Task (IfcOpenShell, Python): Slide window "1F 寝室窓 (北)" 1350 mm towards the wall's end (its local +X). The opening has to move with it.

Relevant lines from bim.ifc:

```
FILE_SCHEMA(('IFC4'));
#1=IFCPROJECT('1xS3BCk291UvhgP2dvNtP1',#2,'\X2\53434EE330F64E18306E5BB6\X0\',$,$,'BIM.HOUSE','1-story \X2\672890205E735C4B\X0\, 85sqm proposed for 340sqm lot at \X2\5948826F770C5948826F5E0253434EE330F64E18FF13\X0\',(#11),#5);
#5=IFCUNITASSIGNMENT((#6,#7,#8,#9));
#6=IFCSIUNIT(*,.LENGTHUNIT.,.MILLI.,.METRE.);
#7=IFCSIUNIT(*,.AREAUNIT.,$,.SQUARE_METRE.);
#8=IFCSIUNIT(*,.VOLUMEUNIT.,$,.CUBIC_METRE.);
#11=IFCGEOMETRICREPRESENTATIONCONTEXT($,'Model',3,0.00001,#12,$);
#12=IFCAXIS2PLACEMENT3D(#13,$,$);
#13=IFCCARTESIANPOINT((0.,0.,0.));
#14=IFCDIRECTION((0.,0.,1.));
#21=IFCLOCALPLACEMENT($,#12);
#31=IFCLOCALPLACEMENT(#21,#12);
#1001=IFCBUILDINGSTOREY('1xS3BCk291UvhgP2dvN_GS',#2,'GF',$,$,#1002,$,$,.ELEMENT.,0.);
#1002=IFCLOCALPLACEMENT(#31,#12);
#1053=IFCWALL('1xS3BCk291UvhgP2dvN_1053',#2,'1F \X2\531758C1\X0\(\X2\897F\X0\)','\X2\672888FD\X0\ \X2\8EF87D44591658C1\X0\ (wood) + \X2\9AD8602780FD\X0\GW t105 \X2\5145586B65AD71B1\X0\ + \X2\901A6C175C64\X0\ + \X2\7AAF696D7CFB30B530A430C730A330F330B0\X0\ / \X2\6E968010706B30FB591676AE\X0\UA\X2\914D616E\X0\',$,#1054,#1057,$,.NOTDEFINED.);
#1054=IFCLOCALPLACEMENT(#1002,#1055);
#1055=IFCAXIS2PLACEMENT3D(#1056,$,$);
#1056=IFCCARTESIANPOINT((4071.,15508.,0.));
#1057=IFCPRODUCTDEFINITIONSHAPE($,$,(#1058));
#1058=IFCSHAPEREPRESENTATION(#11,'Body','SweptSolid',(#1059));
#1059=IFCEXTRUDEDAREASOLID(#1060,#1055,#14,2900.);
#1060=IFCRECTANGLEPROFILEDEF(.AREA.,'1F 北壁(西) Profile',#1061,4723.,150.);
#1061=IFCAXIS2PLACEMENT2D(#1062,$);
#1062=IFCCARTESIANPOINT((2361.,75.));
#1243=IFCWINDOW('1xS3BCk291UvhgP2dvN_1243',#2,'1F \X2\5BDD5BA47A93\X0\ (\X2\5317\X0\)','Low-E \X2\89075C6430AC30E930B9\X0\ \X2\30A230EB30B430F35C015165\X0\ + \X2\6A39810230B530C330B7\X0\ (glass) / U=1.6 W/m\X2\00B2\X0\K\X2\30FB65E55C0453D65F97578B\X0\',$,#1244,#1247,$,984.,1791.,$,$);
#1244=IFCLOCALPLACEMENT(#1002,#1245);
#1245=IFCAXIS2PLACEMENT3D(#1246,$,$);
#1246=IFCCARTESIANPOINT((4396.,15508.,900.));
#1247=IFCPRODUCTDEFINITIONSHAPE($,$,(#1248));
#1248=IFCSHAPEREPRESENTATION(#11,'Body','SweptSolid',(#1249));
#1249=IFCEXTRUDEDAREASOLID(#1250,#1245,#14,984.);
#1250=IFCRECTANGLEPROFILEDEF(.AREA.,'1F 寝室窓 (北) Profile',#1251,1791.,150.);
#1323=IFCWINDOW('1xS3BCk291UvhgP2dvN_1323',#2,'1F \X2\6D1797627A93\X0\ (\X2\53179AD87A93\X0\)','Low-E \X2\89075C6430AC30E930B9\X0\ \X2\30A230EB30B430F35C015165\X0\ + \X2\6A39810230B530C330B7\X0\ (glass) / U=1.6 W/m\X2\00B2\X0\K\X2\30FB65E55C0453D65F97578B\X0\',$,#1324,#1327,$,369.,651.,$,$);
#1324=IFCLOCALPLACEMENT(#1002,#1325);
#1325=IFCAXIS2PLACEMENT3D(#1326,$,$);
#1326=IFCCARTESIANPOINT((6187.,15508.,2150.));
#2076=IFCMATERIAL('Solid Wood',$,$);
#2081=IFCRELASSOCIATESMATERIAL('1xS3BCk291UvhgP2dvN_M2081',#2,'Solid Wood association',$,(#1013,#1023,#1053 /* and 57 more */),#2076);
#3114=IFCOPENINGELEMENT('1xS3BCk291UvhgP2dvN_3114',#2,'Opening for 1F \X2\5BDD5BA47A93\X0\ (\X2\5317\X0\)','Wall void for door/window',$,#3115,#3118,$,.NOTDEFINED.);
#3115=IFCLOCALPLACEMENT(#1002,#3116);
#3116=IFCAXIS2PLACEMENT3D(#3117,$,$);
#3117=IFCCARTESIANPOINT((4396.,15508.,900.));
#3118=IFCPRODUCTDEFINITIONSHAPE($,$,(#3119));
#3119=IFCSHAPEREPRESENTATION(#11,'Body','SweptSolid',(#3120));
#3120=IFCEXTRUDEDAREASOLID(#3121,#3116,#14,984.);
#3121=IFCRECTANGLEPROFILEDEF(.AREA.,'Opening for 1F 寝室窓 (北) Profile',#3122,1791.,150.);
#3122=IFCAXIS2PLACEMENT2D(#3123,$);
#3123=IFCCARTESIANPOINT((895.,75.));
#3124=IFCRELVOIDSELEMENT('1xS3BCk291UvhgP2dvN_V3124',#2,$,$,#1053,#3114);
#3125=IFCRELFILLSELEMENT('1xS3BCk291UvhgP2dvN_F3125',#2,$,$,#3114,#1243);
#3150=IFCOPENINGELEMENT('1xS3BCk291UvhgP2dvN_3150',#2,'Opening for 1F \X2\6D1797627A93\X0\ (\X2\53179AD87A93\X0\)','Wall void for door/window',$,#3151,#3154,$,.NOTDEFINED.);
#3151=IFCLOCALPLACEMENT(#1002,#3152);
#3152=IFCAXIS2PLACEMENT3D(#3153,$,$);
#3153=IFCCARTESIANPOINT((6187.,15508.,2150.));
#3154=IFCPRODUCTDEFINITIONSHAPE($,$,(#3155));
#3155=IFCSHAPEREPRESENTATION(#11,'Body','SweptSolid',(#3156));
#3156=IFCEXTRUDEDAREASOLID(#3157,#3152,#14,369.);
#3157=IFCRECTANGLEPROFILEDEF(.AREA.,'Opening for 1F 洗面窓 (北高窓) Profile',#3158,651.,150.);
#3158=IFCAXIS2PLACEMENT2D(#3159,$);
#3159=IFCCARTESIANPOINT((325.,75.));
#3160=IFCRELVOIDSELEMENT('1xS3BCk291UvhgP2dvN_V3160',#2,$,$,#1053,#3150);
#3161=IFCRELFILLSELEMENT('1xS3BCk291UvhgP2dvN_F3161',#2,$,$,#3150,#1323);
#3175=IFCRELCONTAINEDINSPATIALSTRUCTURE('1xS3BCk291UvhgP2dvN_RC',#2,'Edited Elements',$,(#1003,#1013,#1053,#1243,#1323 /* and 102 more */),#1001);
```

```python
import ifcopenshell
import ifcopenshell.api.geometry
import ifcopenshell.util.placement
import ifcopenshell.util.unit

model = ifcopenshell.open("bim.ifc")
unit_scale = ifcopenshell.util.unit.calculate_unit_scale(model)

window = model.by_guid("1xS3BCk291UvhgP2dvN_1243")
opening = window.FillsVoids[0].RelatingOpeningElement
wall = opening.VoidsElements[0].RelatingBuildingElement

wall_matrix = ifcopenshell.util.placement.get_local_placement(wall.ObjectPlacement)
shift = wall_matrix[:3, 0] * 1.35 / unit_scale
before = ifcopenshell.util.placement.get_local_placement(window.ObjectPlacement)[:3, 3].copy()

# The window is not placed relative to its opening, so move both.
for product in (opening, window):
    matrix = ifcopenshell.util.placement.get_local_placement(product.ObjectPlacement)
    matrix[:3, 3] += shift
    ifcopenshell.api.geometry.edit_object_placement(model, product=product, matrix=matrix, is_si=False)

after = ifcopenshell.util.placement.get_local_placement(window.ObjectPlacement)[:3, 3]
print("window moved by", (after - before).round(3) + 0.0)

model.write("bim_v2.ifc")
```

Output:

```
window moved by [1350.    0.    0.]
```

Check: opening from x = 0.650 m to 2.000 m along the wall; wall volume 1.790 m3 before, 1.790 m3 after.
